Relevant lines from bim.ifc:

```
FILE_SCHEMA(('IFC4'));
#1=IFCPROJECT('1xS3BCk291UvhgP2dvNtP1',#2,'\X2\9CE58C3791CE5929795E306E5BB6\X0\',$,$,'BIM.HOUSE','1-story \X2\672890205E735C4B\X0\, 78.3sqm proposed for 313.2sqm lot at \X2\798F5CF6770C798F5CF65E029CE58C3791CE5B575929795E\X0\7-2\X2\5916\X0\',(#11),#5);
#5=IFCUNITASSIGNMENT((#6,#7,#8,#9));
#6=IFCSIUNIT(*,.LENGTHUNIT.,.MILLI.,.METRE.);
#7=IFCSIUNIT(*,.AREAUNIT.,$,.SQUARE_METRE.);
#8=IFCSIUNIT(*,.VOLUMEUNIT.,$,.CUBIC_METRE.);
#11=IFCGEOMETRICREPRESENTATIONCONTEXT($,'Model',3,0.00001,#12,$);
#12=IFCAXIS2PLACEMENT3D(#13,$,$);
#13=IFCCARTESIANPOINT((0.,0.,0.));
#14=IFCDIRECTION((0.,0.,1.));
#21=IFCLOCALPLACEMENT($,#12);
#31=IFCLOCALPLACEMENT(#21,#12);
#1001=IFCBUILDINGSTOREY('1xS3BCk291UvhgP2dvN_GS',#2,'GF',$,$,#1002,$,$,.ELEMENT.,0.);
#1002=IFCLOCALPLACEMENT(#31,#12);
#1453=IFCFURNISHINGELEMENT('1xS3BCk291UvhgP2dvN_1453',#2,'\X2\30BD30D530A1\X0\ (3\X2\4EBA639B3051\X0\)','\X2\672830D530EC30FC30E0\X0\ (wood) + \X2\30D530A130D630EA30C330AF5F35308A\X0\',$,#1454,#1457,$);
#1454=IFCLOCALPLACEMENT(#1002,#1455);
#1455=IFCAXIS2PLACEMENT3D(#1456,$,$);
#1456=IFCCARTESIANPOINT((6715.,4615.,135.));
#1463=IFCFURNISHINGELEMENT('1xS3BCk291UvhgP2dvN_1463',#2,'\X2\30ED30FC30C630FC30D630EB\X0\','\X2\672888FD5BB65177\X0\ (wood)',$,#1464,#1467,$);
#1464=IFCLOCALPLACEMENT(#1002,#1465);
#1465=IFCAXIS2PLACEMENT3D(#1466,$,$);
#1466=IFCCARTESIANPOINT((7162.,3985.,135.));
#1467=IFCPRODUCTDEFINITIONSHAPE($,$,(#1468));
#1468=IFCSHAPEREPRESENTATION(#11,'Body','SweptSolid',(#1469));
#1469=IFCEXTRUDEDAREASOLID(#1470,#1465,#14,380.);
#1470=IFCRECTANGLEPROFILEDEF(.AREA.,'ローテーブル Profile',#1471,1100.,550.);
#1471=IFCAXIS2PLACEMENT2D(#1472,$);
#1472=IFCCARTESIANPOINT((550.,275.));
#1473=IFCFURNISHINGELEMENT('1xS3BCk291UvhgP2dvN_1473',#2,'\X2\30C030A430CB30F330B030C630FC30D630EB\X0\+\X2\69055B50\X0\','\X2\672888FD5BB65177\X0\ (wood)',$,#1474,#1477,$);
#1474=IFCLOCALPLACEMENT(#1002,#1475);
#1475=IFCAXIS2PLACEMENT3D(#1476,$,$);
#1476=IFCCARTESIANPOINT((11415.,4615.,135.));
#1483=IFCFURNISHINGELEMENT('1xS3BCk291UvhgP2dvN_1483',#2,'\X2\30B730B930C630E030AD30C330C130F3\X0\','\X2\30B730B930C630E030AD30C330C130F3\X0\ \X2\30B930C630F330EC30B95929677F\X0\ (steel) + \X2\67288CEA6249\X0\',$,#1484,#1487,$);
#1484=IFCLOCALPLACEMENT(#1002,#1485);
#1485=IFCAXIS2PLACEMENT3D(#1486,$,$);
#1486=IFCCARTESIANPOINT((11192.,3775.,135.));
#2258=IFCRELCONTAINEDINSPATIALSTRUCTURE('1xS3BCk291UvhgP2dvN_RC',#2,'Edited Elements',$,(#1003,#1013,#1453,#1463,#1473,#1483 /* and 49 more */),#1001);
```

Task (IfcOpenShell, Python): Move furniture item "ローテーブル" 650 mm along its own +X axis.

```python
import ifcopenshell
import ifcopenshell.api.geometry
import ifcopenshell.util.placement

model = ifcopenshell.open("bim.ifc")

item = model.by_guid("1xS3BCk291UvhgP2dvN_1463")
matrix = ifcopenshell.util.placement.get_local_placement(item.ObjectPlacement)
matrix[:3, 3] += matrix[:3, 0] * 650.0
ifcopenshell.api.geometry.edit_object_placement(model, product=item, matrix=matrix, is_si=False)

print(ifcopenshell.util.placement.get_local_placement(item.ObjectPlacement).round(3) + 0.0)

model.write("bim-out.ifc")
```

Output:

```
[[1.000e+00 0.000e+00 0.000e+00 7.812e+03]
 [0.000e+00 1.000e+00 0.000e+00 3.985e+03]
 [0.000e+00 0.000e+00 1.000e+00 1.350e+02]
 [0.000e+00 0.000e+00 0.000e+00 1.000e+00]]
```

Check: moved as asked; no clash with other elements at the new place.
